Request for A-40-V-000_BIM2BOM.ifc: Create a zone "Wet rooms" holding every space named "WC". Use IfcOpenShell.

First a look at what the model holds.

```python
import ifcopenshell

model = ifcopenshell.open("A-40-V-000_BIM2BOM.ifc")
print(model.schema)
seen = {}
for space in model.by_type("IfcSpace"):
    seen[space.LongName] = seen.get(space.LongName, 0) + 1
for name, count in sorted(seen.items(), key=str):
    print(count, "x", name)
print("zones:", [z.Name for z in model.by_type("IfcZone")][:20])
```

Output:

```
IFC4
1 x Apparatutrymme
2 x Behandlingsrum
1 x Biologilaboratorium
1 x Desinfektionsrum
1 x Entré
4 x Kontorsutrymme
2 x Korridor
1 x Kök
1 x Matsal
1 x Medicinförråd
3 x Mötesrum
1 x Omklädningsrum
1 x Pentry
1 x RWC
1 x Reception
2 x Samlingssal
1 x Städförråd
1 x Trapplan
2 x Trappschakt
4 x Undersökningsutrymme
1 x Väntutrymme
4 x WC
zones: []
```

```python
import ifcopenshell
import ifcopenshell.api.group
import ifcopenshell.api.root

model = ifcopenshell.open("A-40-V-000_BIM2BOM.ifc")

names = {"WC"}
spaces = [s for s in model.by_type("IfcSpace") if s.LongName in names]

zone = ifcopenshell.api.root.create_entity(model, ifc_class="IfcZone", name="Wet rooms")
ifcopenshell.api.group.assign_group(model, products=spaces, group=zone)
print(len(spaces), "spaces in", zone.Name)

model.write("A-40-V-000_BIM2BOM_edited.ifc")
```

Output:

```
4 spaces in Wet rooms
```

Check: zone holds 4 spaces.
